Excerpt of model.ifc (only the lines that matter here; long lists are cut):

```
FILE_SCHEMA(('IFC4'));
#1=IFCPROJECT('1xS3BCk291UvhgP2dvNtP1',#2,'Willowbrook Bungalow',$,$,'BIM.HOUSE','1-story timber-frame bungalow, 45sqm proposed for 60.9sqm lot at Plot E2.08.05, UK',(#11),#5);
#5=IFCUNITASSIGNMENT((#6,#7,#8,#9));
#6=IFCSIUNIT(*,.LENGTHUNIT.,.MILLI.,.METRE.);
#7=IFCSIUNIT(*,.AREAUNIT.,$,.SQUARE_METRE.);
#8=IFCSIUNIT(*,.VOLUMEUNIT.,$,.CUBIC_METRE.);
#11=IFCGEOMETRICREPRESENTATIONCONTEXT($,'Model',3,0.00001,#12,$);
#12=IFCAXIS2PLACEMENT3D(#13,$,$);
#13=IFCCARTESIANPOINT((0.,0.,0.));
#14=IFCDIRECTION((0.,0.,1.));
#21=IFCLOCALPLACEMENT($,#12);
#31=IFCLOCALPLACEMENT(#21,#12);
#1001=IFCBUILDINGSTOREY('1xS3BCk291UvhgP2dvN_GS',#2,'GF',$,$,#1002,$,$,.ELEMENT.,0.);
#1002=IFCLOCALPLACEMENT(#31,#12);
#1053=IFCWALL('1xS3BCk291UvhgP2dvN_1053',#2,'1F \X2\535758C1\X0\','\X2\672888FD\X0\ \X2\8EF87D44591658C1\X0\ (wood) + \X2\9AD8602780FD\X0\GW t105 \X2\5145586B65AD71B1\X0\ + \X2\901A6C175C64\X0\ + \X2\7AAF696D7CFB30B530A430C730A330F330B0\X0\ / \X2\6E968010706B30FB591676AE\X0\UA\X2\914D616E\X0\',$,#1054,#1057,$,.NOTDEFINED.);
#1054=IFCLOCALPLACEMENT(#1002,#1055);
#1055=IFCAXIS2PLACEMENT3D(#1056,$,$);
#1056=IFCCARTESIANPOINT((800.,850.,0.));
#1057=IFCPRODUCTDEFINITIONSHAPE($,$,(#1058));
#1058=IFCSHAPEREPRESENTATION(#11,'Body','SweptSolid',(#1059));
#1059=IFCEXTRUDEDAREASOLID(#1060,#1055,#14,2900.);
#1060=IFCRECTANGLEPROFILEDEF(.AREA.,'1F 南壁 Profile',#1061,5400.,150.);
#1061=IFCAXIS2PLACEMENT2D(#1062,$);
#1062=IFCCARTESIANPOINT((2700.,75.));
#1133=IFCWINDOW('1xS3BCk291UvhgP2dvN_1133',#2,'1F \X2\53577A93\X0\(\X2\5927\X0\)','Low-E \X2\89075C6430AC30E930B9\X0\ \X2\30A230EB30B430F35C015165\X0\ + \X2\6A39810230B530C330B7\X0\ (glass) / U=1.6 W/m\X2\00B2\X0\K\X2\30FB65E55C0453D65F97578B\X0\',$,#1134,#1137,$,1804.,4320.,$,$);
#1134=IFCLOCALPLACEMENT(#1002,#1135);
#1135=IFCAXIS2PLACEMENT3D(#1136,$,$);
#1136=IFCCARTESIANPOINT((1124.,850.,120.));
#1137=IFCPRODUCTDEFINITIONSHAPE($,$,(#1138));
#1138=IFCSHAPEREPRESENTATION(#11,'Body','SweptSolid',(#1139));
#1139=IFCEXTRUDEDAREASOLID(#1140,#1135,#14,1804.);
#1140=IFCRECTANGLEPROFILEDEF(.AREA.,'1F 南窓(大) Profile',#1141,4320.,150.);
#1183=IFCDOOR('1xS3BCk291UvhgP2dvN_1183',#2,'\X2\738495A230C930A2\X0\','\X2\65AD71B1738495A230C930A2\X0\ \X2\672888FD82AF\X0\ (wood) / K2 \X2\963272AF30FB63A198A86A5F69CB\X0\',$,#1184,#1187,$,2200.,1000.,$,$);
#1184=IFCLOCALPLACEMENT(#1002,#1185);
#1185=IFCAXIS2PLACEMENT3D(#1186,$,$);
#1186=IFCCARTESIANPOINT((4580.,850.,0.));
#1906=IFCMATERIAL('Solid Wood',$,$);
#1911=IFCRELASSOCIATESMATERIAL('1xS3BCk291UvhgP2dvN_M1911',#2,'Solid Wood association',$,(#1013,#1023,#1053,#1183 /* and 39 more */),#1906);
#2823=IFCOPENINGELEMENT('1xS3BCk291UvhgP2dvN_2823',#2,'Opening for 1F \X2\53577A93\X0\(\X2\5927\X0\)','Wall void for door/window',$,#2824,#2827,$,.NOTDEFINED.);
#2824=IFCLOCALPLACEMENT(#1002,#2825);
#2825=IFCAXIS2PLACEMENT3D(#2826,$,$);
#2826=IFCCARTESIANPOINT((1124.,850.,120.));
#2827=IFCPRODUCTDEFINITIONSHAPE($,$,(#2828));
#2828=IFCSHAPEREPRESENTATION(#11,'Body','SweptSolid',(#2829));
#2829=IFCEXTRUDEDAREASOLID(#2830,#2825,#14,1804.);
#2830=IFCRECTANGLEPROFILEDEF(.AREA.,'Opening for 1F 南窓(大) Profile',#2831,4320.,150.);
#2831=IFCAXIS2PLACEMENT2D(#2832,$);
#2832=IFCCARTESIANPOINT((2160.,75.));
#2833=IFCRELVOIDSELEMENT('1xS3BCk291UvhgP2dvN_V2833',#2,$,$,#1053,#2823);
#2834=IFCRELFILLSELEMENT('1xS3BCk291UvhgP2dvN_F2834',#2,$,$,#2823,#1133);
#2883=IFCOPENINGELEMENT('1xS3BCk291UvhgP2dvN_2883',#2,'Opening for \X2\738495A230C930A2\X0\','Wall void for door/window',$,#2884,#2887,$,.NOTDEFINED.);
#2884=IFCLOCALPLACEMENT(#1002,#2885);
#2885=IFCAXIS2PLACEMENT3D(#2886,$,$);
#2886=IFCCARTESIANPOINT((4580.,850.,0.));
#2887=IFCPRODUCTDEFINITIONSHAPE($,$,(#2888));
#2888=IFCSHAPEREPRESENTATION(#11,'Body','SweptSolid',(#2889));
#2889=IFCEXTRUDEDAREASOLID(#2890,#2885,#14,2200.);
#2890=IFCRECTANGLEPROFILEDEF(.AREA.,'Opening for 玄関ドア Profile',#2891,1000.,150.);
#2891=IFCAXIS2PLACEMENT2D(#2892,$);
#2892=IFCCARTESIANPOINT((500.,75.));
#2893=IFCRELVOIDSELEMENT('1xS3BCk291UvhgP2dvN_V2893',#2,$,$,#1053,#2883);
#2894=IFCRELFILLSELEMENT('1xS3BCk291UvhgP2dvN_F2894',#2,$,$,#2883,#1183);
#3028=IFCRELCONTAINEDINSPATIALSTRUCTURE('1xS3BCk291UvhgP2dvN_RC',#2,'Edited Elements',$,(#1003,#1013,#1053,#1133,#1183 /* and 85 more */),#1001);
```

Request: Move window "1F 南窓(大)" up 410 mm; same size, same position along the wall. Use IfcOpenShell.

```python
import numpy as np
import ifcopenshell
import ifcopenshell.api.geometry
import ifcopenshell.util.placement
import ifcopenshell.util.unit

model = ifcopenshell.open("model.ifc")
unit_scale = ifcopenshell.util.unit.calculate_unit_scale(model)

window = model.by_id(1133)
opening = window.FillsVoids[0].RelatingOpeningElement
dz = 410.0

shift = np.array([0.0, 0.0, dz])
# The window is not placed relative to its opening, so move both.
for product in (opening, window):
    matrix = ifcopenshell.util.placement.get_local_placement(product.ObjectPlacement)
    matrix[:3, 3] += shift
    ifcopenshell.api.geometry.edit_object_placement(model, product=product, matrix=matrix, is_si=False)

print(f"moved by {dz * unit_scale:+.3f} m")

model.write("model_v2.ifc")
```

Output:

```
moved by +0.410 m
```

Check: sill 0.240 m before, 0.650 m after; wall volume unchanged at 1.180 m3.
